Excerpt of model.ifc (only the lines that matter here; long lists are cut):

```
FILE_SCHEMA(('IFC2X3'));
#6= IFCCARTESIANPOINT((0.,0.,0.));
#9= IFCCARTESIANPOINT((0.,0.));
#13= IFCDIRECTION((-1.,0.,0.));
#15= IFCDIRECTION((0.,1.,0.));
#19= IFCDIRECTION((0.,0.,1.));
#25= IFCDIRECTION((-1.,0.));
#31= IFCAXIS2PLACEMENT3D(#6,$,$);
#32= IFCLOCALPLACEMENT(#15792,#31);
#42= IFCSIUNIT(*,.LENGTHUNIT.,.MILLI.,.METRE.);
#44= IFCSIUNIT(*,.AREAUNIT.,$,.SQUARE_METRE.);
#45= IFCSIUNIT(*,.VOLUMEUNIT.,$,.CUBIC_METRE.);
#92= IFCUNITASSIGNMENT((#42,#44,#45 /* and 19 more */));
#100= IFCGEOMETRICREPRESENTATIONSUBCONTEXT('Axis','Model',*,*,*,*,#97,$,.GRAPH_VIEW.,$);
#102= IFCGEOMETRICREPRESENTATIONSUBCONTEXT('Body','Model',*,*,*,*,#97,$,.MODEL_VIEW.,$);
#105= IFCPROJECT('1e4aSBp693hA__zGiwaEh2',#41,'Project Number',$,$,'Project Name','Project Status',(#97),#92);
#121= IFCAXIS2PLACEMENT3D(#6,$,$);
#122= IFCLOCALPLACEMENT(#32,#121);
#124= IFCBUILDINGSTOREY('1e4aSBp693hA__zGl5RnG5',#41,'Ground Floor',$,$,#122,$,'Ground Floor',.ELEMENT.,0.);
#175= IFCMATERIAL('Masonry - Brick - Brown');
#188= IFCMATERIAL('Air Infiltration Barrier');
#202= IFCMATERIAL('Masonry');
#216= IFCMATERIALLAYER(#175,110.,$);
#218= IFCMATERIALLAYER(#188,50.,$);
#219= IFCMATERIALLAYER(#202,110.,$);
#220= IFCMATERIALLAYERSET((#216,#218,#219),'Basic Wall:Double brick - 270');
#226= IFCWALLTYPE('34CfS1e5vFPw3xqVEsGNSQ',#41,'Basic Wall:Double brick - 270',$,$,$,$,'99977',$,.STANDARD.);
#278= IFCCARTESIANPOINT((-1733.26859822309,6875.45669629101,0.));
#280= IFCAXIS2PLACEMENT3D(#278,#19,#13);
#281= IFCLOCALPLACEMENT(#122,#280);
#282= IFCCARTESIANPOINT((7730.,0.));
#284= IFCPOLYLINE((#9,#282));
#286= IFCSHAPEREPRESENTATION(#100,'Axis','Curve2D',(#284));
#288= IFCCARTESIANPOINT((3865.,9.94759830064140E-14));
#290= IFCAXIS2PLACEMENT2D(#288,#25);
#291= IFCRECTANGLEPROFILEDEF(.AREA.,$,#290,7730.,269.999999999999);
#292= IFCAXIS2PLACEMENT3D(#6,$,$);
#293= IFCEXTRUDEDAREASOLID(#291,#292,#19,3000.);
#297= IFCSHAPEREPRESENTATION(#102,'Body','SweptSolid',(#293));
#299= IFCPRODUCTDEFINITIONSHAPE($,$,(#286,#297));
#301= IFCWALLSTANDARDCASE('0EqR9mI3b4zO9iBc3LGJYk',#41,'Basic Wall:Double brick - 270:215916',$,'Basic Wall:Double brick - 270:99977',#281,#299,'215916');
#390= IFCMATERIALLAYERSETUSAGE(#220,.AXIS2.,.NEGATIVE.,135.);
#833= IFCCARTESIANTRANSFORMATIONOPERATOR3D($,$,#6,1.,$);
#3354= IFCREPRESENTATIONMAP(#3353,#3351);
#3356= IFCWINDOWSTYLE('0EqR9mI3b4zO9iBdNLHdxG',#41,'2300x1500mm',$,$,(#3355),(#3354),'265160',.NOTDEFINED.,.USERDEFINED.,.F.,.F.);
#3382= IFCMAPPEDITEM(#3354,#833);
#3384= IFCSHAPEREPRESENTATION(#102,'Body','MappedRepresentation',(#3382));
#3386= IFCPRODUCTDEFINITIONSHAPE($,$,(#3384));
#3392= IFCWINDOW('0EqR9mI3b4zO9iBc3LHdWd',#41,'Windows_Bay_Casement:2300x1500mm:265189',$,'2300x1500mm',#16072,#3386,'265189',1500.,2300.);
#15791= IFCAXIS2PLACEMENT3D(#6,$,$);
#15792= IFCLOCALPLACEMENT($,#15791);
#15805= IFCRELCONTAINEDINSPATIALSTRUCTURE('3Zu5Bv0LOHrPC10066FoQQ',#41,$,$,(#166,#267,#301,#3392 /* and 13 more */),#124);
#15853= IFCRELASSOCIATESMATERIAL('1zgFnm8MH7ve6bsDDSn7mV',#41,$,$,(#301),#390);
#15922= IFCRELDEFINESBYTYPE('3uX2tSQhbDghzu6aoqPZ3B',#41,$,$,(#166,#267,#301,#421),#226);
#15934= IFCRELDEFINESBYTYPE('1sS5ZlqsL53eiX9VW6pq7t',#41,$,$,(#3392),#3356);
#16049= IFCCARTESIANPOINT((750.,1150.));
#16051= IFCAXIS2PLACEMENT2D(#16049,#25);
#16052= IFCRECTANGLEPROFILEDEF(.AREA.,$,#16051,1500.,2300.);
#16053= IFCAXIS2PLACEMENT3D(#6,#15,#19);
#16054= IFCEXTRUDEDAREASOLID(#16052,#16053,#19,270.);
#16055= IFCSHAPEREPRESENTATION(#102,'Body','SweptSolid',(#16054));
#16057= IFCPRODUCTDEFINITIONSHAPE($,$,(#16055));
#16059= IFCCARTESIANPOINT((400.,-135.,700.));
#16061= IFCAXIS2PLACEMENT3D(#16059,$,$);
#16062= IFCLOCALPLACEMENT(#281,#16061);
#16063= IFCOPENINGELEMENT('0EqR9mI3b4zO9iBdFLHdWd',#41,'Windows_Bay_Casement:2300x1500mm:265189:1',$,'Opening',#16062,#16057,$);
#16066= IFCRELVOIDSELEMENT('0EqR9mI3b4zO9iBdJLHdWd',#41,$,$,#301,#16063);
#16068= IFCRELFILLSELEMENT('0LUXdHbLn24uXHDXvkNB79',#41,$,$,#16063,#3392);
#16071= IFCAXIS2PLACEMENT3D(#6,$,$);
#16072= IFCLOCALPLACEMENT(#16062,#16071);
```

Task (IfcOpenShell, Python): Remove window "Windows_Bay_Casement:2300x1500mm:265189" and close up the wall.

```python
import ifcopenshell
import ifcopenshell.api.feature
import ifcopenshell.api.root
import ifcopenshell.geom
import ifcopenshell.util.shape

model = ifcopenshell.open("model.ifc")
settings = ifcopenshell.geom.settings()


def volume(element):
    """Net volume in cubic metres, openings subtracted."""
    shape = ifcopenshell.geom.create_shape(settings, element)
    return ifcopenshell.util.shape.get_volume(shape.geometry)


window = model.by_guid("0EqR9mI3b4zO9iBc3LHdWd")
opening = window.FillsVoids[0].RelatingOpeningElement
wall = opening.VoidsElements[0].RelatingBuildingElement
before = volume(wall)

ifcopenshell.api.root.remove_product(model, product=window)
ifcopenshell.api.feature.remove_feature(model, feature=opening)

after = volume(wall)

print(f"wall volume {before:.3f} -> {after:.3f} m3")

model.write("model_edited.ifc")
```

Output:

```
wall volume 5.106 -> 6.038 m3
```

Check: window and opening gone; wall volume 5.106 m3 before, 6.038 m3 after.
